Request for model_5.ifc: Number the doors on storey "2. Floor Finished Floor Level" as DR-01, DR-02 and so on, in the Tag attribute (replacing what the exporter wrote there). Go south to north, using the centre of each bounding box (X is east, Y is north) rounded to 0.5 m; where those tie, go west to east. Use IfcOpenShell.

First a look at what the model holds.

```python
import ifcopenshell
import ifcopenshell.util.element
import ifcopenshell.util.placement

model = ifcopenshell.open("model_5.ifc")
print(model.schema)
storey = next(s for s in model.by_type("IfcBuildingStorey") if s.Name == "2. Floor Finished Floor Level")
doors = [e for e in ifcopenshell.util.element.get_decomposition(storey) if e.is_a("IfcDoor")]
for e in sorted(doors, key=lambda e: e.id()):
    origin = ifcopenshell.util.placement.get_local_placement(e.ObjectPlacement)[:3, 3]
    print(e.id(), e.Tag, e.Name, origin.round(2) + 0.0, sep=" | ")
```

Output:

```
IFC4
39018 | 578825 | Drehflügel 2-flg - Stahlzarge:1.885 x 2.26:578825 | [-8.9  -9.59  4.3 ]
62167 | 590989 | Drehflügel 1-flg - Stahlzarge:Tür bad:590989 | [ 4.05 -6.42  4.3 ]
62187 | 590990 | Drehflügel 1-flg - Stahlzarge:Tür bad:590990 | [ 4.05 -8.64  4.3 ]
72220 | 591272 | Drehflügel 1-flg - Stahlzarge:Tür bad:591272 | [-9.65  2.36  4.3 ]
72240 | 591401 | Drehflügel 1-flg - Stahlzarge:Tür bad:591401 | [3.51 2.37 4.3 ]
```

```python
import ifcopenshell
import ifcopenshell.geom
import ifcopenshell.util.element
import ifcopenshell.util.shape

model = ifcopenshell.open("model_5.ifc")
settings = ifcopenshell.geom.settings()
settings.set("use-world-coords", True)


def centre(element):
    shape = ifcopenshell.geom.create_shape(settings, element)
    return ifcopenshell.util.shape.get_bbox_centroid(shape.geometry)


storey = next(s for s in model.by_type("IfcBuildingStorey") if s.Name == "2. Floor Finished Floor Level")
doors = [e for e in ifcopenshell.util.element.get_decomposition(storey) if e.is_a("IfcDoor")]

# Insertion points can sit at a corner or the storey origin, so sort by the geometry (in metres).
centres = {e: centre(e) for e in doors}
doors.sort(key=lambda e: (round(centres[e][1] / 0.5), centres[e][0]))

for i, e in enumerate(doors, start=1):
    number = f"DR-{i:02d}"
    e.Tag = number
    print(e.id(), number)

model.write("model_5_updated.ifc")
```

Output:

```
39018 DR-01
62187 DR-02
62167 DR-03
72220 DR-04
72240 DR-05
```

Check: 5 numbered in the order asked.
